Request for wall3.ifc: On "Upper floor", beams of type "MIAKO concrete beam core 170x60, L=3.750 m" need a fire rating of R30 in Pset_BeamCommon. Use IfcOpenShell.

First a look at what the model holds.

```python
import ifcopenshell
import ifcopenshell.util.element

model = ifcopenshell.open("wall3.ifc")
print(model.schema)
storey = next(s for s in model.by_type("IfcBuildingStorey") if s.Name == "Upper floor")
beams = [e for e in ifcopenshell.util.element.get_decomposition(storey) if e.is_a("IfcBeam")]
seen = {}
for e in beams:
    element_type = ifcopenshell.util.element.get_type(e)
    key = (element_type.Name if element_type != e and element_type else None, ifcopenshell.util.element.get_pset(e, "Pset_BeamCommon", "FireRating"))
    seen[key] = seen.get(key, 0) + 1
for (name, value), count in sorted(seen.items(), key=str):
    print(count, "x", name, "|", value)
```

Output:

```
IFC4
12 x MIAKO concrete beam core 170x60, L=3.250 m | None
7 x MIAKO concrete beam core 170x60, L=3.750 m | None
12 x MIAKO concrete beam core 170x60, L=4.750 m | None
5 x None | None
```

```python
import ifcopenshell
import ifcopenshell.api.pset
import ifcopenshell.util.element

model = ifcopenshell.open("wall3.ifc")

storey = next(s for s in model.by_type("IfcBuildingStorey") if s.Name == "Upper floor")
beams = [e for e in ifcopenshell.util.element.get_decomposition(storey) if e.is_a("IfcBeam")]

count = 0
for e in beams:
    element_type = ifcopenshell.util.element.get_type(e)
    if element_type in (None, e) or element_type.Name != "MIAKO concrete beam core 170x60, L=3.750 m":
        continue
    # add_pset returns the element's existing set when there is one.
    pset = ifcopenshell.api.pset.add_pset(model, product=e, name="Pset_BeamCommon")
    ifcopenshell.api.pset.edit_pset(model, pset=pset, properties={"FireRating": "R30"})
    count += 1

print(count, "beams updated")

model.write("wall3_v2.ifc")
```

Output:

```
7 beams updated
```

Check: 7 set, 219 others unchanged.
